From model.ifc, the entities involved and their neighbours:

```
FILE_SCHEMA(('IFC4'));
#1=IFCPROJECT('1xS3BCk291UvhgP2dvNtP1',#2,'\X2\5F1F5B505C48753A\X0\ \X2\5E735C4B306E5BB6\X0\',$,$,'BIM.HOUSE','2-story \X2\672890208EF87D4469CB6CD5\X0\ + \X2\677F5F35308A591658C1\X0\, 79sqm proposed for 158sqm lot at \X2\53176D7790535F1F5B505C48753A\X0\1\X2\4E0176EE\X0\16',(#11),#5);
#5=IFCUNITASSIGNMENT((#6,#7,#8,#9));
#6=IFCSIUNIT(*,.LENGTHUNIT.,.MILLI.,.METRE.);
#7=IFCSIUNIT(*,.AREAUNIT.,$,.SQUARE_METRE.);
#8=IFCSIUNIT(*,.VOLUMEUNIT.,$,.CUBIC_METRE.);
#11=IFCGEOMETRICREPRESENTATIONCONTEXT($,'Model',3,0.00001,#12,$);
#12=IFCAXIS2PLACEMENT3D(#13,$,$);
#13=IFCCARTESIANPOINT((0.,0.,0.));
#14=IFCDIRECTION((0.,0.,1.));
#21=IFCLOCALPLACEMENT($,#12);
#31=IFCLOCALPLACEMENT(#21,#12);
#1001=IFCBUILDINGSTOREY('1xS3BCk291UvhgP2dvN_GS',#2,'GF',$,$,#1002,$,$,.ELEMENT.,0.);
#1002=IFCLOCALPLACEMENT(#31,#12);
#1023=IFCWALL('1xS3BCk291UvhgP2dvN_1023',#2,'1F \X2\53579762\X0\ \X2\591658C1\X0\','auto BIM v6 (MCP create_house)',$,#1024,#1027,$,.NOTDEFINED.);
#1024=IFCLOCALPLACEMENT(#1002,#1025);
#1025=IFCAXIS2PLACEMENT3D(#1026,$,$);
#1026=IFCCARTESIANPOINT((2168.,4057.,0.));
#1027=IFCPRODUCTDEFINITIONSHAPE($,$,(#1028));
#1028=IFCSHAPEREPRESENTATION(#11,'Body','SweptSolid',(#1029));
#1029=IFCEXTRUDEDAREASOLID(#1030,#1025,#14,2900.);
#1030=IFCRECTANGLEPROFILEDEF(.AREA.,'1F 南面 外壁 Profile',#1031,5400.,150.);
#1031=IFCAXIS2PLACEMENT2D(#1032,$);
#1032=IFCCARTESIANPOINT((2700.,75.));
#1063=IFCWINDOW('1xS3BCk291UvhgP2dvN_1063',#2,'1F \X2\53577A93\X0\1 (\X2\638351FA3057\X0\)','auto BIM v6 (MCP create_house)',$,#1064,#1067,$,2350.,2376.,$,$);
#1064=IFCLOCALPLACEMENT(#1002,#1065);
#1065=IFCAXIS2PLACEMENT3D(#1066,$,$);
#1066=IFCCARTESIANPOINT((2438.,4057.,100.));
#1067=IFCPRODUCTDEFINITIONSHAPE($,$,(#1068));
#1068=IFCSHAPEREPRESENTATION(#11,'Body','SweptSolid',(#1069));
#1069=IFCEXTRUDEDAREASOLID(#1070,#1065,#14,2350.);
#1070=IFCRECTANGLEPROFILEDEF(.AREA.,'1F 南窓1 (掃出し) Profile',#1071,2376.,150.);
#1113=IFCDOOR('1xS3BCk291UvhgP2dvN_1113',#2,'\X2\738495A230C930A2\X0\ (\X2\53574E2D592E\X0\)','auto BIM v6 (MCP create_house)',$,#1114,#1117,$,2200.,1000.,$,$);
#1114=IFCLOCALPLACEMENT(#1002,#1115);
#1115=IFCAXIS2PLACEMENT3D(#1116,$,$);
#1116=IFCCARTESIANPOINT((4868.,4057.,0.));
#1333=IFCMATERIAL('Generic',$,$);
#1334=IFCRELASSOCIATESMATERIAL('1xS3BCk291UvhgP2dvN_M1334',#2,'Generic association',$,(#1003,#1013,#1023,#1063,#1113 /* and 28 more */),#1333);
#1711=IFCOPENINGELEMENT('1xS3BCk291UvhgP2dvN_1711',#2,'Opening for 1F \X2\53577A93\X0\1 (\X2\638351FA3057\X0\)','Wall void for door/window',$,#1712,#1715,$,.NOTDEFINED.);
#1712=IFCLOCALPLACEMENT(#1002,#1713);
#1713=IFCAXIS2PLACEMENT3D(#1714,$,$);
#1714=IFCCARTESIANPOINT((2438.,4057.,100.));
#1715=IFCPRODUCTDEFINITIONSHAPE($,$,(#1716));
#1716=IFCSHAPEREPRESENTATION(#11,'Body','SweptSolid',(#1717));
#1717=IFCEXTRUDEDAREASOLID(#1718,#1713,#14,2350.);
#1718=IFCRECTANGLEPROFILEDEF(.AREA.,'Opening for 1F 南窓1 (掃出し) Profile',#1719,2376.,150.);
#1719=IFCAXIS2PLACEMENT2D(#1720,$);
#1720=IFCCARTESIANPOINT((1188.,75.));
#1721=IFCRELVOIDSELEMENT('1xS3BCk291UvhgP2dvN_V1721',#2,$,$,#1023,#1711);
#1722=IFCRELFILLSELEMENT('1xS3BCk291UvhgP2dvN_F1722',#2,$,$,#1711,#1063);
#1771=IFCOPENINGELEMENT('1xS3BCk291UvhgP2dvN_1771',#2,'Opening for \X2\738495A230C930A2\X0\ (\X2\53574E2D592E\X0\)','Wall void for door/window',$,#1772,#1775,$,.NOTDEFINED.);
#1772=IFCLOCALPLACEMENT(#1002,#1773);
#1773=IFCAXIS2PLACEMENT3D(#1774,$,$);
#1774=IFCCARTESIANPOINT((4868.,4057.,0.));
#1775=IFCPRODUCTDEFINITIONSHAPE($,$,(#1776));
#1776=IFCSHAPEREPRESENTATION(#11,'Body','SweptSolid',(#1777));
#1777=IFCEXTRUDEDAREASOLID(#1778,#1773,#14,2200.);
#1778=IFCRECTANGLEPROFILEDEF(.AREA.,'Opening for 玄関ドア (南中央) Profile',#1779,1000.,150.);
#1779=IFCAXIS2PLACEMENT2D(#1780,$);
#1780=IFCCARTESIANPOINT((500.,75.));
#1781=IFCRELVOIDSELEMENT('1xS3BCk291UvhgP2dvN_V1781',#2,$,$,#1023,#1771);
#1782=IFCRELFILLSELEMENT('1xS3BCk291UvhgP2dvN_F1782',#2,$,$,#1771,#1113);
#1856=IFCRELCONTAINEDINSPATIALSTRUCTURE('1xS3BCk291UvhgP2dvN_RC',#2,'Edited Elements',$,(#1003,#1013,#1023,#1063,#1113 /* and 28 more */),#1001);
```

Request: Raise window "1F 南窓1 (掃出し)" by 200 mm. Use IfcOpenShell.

```python
import numpy as np
import ifcopenshell
import ifcopenshell.api.geometry
import ifcopenshell.util.placement
import ifcopenshell.util.unit

model = ifcopenshell.open("model.ifc")
unit_scale = ifcopenshell.util.unit.calculate_unit_scale(model)

window = model.by_guid("1xS3BCk291UvhgP2dvN_1063")
opening = window.FillsVoids[0].RelatingOpeningElement
dz = 200.0

shift = np.array([0.0, 0.0, dz])
# The window is not placed relative to its opening, so move both.
for product in (opening, window):
    matrix = ifcopenshell.util.placement.get_local_placement(product.ObjectPlacement)
    matrix[:3, 3] += shift
    ifcopenshell.api.geometry.edit_object_placement(model, product=product, matrix=matrix, is_si=False)

print(f"moved by {dz * unit_scale:+.3f} m")

model.write("model_updated.ifc")
```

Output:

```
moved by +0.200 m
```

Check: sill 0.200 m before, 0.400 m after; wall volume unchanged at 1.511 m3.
